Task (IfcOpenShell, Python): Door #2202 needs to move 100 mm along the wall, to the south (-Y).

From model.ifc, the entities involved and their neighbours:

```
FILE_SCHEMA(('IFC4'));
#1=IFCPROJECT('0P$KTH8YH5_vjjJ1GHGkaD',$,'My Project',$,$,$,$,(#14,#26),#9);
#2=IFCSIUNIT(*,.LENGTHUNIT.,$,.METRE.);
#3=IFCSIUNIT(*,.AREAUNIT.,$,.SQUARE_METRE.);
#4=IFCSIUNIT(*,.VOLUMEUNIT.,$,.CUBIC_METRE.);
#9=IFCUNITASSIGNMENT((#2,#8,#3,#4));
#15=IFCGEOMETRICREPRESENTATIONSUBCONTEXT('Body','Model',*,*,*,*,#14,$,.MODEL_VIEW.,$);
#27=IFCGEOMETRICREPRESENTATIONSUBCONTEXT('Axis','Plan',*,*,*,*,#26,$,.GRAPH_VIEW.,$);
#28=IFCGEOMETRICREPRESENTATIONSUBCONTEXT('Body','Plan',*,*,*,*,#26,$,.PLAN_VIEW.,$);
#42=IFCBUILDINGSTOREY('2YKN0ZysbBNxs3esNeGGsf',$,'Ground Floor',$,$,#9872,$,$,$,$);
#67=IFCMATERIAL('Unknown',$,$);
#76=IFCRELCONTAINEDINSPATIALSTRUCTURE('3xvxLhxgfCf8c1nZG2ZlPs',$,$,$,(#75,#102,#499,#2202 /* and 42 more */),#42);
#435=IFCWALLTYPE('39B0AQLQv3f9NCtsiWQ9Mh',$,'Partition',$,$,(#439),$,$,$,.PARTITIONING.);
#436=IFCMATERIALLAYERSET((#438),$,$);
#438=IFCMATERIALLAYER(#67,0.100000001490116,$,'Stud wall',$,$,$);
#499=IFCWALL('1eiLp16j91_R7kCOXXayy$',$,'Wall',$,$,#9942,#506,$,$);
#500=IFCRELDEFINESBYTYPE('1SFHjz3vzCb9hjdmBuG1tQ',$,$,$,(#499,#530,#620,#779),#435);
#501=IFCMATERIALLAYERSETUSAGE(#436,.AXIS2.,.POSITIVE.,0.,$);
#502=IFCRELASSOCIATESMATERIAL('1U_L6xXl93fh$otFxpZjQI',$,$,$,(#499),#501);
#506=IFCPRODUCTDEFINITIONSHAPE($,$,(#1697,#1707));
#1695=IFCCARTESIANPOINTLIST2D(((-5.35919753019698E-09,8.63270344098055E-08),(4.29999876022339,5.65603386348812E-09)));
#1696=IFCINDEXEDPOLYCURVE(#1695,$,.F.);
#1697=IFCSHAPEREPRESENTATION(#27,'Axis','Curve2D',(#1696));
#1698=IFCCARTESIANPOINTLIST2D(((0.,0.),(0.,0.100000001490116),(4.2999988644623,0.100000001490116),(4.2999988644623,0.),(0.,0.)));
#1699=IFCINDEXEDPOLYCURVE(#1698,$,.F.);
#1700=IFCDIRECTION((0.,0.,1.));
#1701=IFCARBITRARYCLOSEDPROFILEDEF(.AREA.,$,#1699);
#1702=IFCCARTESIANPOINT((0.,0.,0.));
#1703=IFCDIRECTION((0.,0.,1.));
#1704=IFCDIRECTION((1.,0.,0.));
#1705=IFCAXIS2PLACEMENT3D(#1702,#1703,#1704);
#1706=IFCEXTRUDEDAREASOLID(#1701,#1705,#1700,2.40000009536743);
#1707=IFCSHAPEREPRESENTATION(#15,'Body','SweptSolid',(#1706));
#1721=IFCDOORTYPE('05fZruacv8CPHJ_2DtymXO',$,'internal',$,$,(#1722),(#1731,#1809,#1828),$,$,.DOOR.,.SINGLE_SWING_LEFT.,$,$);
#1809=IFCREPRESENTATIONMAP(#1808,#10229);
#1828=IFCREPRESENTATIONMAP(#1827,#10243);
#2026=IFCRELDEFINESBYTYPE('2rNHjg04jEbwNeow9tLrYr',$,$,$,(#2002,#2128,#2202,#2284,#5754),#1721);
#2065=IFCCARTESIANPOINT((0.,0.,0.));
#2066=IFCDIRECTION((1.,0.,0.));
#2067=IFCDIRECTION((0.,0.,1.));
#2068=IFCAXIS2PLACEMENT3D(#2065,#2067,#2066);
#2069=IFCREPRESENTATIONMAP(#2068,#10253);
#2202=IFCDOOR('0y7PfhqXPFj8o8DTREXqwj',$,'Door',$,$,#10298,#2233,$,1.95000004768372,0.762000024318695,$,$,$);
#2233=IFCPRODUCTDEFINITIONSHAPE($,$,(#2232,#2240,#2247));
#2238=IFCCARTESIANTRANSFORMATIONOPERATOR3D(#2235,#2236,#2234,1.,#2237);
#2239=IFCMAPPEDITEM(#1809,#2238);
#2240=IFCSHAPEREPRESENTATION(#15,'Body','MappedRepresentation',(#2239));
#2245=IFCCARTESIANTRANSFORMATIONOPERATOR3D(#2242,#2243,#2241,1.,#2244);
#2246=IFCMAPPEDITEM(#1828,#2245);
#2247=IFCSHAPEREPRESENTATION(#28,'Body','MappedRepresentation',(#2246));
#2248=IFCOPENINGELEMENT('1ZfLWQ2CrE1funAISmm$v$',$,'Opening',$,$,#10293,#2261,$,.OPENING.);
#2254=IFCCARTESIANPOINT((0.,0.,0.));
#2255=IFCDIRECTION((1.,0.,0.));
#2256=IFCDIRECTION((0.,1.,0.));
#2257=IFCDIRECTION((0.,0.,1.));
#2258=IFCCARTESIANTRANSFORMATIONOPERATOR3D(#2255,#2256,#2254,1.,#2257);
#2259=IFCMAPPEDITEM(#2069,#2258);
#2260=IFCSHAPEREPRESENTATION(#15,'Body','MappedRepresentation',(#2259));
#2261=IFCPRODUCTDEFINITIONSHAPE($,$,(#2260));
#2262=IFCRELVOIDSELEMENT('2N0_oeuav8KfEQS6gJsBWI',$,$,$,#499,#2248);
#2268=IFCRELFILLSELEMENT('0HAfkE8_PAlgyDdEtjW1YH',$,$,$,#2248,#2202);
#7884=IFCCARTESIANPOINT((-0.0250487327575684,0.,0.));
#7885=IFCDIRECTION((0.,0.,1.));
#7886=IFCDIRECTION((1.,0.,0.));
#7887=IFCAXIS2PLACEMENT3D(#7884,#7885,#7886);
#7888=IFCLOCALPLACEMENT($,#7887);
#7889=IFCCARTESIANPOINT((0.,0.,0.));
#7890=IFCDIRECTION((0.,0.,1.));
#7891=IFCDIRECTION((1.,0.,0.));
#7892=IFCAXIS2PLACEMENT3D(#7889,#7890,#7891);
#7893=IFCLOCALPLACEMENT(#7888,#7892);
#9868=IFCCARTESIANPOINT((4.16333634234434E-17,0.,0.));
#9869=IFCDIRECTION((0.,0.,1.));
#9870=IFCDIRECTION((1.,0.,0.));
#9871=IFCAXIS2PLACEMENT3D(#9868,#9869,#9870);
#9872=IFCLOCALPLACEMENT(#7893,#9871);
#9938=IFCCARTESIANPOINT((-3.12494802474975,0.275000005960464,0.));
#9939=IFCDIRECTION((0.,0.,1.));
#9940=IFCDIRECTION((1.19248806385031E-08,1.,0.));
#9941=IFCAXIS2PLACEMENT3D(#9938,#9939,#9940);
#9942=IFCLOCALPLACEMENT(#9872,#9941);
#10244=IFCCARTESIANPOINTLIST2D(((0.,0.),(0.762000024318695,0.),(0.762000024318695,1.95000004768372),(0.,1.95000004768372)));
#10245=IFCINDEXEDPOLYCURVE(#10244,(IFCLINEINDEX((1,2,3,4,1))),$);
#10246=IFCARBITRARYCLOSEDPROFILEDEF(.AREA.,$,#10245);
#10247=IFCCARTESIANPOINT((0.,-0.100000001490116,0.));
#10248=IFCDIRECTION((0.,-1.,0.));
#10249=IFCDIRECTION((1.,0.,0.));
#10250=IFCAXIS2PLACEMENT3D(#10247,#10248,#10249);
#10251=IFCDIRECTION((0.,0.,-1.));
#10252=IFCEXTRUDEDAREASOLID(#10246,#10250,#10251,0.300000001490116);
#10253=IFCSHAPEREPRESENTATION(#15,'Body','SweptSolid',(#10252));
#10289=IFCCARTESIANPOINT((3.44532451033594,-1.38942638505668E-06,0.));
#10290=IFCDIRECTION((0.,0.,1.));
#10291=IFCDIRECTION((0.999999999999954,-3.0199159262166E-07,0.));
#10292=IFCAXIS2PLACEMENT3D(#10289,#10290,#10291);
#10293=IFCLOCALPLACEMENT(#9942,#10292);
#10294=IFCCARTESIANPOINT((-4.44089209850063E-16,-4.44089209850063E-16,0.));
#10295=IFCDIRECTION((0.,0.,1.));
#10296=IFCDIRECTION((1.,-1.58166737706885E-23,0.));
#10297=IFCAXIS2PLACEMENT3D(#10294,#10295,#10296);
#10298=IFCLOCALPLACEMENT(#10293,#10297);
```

```python
import ifcopenshell
import ifcopenshell.api.geometry
import ifcopenshell.util.placement

model = ifcopenshell.open("model.ifc")

door = model.by_guid("0y7PfhqXPFj8o8DTREXqwj")
opening = door.FillsVoids[0].RelatingOpeningElement
wall = opening.VoidsElements[0].RelatingBuildingElement

wall_matrix = ifcopenshell.util.placement.get_local_placement(wall.ObjectPlacement)
shift = wall_matrix[:3, 0] * -0.1
before = ifcopenshell.util.placement.get_local_placement(door.ObjectPlacement)[:3, 3].copy()

# The door is placed relative to its opening, so it follows when the opening moves.
matrix = ifcopenshell.util.placement.get_local_placement(opening.ObjectPlacement)
matrix[:3, 3] += shift
ifcopenshell.api.geometry.edit_object_placement(
    model, product=opening, matrix=matrix, is_si=False, should_transform_children=True
)

after = ifcopenshell.util.placement.get_local_placement(door.ObjectPlacement)[:3, 3]
print("door moved by", (after - before).round(3) + 0.0)

model.write("model_updated.ifc")
```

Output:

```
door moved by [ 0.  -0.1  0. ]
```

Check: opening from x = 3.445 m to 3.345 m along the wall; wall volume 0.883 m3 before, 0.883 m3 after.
